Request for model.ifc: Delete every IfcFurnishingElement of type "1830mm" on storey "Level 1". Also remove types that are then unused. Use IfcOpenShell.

First a look at what the model holds.

```python
import ifcopenshell
import ifcopenshell.util.element

model = ifcopenshell.open("model.ifc")
print(model.schema)
storey = next(s for s in model.by_type("IfcBuildingStorey") if s.Name == "Level 1")
furniture = [e for e in ifcopenshell.util.element.get_decomposition(storey) if e.is_a("IfcFurnishingElement")]
seen = {}
for e in furniture:
    element_type = ifcopenshell.util.element.get_type(e)
    name = element_type.Name if element_type not in (None, e) else None
    seen[name] = seen.get(name, 0) + 1
for name, count in sorted(seen.items(), key=str):
    print(count, "x", name)
```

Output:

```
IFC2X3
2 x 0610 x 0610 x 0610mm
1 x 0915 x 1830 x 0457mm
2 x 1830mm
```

```python
import ifcopenshell
import ifcopenshell.api.root
import ifcopenshell.util.element

model = ifcopenshell.open("model.ifc")

storey = next(s for s in model.by_type("IfcBuildingStorey") if s.Name == "Level 1")
furniture = [e for e in ifcopenshell.util.element.get_decomposition(storey) if e.is_a("IfcFurnishingElement")]
targets = [e for e in furniture if (t := ifcopenshell.util.element.get_type(e)) not in (None, e) and t.Name == "1830mm"]
types = {ifcopenshell.util.element.get_type(e) for e in targets} - {None, *targets}

for e in targets:
    ifcopenshell.api.root.remove_product(model, product=e)
print(len(targets), "removed")

unused = [t for t in types if not ifcopenshell.util.element.get_types(t)]
for t in unused:
    ifcopenshell.api.root.remove_product(model, product=t)
print(len(unused), "unused types removed")

model.write("model_v2.ifc")
```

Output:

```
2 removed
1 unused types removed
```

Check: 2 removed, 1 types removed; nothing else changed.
